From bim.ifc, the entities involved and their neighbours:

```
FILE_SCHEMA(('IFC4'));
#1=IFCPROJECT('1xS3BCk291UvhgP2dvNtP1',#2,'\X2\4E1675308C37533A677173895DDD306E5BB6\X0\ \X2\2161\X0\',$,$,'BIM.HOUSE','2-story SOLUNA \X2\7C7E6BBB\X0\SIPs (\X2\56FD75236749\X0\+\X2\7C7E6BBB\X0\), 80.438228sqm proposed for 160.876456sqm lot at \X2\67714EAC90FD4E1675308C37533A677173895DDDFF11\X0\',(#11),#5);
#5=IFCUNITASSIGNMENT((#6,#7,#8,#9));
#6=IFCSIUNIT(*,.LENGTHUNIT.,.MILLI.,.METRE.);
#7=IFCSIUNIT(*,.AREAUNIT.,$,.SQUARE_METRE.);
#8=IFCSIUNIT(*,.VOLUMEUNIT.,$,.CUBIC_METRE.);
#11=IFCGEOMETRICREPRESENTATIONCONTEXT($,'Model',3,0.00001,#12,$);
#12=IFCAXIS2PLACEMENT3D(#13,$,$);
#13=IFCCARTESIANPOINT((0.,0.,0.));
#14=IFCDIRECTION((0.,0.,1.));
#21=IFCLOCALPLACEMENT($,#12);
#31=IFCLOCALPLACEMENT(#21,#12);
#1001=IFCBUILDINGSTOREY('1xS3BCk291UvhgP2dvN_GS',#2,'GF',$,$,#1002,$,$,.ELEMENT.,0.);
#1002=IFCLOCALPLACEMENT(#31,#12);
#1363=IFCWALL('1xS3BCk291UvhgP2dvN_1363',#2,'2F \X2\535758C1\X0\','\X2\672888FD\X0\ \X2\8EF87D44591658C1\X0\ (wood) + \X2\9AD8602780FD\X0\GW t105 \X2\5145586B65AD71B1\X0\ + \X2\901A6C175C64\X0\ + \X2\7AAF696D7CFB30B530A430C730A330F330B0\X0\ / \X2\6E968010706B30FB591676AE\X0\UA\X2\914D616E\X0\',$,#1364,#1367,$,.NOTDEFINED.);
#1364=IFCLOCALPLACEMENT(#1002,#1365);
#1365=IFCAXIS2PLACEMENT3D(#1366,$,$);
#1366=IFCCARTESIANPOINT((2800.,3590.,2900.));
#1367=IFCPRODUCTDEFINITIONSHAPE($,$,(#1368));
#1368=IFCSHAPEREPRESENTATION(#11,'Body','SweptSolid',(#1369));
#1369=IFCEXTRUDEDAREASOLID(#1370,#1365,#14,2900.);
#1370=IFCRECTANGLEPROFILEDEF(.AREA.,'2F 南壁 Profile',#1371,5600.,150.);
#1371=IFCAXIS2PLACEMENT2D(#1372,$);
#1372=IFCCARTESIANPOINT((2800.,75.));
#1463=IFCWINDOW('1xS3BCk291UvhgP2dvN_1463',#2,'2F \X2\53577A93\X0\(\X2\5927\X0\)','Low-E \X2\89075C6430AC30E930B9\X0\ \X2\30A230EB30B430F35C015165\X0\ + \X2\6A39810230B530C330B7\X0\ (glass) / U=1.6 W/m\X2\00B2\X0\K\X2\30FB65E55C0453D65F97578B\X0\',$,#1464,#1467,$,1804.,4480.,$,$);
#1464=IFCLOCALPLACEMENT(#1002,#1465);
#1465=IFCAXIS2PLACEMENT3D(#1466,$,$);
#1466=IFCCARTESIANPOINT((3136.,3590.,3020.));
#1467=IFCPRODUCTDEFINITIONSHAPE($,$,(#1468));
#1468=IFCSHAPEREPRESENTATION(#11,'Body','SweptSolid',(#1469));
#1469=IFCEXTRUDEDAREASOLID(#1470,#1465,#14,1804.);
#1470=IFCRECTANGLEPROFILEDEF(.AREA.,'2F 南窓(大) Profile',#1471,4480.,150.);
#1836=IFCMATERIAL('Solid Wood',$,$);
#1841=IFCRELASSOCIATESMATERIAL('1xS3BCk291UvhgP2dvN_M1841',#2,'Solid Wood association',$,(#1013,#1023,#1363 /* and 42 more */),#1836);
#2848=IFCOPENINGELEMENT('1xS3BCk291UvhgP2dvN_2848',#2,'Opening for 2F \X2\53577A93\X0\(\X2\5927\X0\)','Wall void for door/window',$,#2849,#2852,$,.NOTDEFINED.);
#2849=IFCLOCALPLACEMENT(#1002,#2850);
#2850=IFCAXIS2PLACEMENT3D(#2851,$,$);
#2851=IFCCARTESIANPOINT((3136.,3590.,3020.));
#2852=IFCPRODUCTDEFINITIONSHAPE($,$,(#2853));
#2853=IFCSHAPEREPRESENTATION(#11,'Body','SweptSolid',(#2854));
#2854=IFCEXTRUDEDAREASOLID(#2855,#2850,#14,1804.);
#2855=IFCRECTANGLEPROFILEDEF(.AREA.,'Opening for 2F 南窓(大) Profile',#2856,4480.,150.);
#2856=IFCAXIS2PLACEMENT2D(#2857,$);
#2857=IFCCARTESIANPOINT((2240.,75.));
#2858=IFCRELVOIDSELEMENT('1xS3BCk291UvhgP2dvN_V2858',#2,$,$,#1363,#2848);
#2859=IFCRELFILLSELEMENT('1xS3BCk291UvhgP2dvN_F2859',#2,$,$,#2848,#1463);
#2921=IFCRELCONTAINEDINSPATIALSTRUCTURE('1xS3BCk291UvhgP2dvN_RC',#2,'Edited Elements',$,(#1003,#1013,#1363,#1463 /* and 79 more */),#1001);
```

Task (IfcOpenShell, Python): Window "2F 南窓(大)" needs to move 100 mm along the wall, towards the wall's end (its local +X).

```python
import ifcopenshell
import ifcopenshell.api.geometry
import ifcopenshell.util.placement
import ifcopenshell.util.unit

model = ifcopenshell.open("bim.ifc")
unit_scale = ifcopenshell.util.unit.calculate_unit_scale(model)

window = model.by_guid("1xS3BCk291UvhgP2dvN_1463")
opening = window.FillsVoids[0].RelatingOpeningElement
wall = opening.VoidsElements[0].RelatingBuildingElement

wall_matrix = ifcopenshell.util.placement.get_local_placement(wall.ObjectPlacement)
shift = wall_matrix[:3, 0] * 0.1 / unit_scale
before = ifcopenshell.util.placement.get_local_placement(window.ObjectPlacement)[:3, 3].copy()

# The window is not placed relative to its opening, so move both.
for product in (opening, window):
    matrix = ifcopenshell.util.placement.get_local_placement(product.ObjectPlacement)
    matrix[:3, 3] += shift
    ifcopenshell.api.geometry.edit_object_placement(model, product=product, matrix=matrix, is_si=False)

after = ifcopenshell.util.placement.get_local_placement(window.ObjectPlacement)[:3, 3]
print("window moved by", (after - before).round(3) + 0.0)

model.write("bim_updated.ifc")
```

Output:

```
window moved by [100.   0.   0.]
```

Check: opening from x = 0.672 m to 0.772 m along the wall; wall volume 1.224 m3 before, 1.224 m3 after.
